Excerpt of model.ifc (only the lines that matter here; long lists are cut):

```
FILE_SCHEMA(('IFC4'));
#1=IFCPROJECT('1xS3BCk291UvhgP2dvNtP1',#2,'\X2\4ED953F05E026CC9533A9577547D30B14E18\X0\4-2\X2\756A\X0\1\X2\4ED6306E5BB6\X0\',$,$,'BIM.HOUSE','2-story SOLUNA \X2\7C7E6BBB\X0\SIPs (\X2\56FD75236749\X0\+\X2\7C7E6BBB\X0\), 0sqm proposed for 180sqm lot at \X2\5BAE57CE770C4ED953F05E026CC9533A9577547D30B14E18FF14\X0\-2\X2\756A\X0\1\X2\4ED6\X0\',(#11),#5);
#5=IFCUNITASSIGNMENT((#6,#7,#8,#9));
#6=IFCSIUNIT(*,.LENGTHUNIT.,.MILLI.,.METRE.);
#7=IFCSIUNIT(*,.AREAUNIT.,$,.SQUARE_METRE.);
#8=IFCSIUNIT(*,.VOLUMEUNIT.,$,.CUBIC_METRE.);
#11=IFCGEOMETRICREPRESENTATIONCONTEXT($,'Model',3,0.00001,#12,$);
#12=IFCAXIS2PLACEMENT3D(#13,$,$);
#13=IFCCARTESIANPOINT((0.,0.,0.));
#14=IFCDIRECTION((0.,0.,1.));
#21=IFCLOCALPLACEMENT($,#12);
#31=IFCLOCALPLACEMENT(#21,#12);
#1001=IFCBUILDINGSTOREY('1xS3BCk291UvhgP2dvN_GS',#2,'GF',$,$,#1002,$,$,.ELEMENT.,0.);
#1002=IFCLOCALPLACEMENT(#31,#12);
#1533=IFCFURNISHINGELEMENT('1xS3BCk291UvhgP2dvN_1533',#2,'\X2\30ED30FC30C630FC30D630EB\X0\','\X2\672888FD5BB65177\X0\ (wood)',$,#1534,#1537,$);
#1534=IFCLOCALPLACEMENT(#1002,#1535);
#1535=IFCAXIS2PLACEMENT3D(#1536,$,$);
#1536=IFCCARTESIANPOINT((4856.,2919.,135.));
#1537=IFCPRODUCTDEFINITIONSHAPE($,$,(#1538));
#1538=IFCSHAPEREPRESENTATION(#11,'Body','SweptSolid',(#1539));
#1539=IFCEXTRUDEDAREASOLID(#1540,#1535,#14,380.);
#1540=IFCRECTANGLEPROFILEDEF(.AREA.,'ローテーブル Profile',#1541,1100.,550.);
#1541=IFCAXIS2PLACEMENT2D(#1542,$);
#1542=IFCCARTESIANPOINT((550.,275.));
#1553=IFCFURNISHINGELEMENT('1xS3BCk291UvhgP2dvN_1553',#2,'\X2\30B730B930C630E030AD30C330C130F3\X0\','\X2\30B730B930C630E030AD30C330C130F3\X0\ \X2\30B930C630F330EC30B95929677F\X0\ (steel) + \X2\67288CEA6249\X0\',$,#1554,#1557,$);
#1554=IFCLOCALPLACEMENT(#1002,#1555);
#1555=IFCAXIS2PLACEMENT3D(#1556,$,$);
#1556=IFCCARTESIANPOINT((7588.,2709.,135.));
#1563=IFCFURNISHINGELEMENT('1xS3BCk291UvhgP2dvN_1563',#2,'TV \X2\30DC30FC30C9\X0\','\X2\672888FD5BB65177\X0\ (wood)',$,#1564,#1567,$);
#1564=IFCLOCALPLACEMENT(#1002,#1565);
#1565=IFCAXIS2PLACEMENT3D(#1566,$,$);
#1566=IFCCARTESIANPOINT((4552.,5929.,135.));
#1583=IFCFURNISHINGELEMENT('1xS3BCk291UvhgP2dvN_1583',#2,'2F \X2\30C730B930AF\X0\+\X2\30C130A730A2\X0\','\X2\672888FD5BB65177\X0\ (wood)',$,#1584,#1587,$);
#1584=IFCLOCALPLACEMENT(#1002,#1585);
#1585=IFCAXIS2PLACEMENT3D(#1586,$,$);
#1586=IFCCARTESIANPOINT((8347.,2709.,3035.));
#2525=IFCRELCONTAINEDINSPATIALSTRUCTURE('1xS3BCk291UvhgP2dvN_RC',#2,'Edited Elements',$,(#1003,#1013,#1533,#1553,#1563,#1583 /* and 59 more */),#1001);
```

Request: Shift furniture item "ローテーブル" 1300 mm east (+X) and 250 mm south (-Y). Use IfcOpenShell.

```python
import ifcopenshell
import ifcopenshell.api.geometry
import ifcopenshell.util.placement
import ifcopenshell.util.unit

model = ifcopenshell.open("model.ifc")
unit_scale = ifcopenshell.util.unit.calculate_unit_scale(model)

item = model.by_guid("1xS3BCk291UvhgP2dvN_1533")
matrix = ifcopenshell.util.placement.get_local_placement(item.ObjectPlacement)
matrix[0, 3] += 1.3 / unit_scale
matrix[1, 3] -= 0.25 / unit_scale
ifcopenshell.api.geometry.edit_object_placement(model, product=item, matrix=matrix, is_si=False)

print(ifcopenshell.util.placement.get_local_placement(item.ObjectPlacement).round(3) + 0.0)

model.write("model_rev.ifc")
```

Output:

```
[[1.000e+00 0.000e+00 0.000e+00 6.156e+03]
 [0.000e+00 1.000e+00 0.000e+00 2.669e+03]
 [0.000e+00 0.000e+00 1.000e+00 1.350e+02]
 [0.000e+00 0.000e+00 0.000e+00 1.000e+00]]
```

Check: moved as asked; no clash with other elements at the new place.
